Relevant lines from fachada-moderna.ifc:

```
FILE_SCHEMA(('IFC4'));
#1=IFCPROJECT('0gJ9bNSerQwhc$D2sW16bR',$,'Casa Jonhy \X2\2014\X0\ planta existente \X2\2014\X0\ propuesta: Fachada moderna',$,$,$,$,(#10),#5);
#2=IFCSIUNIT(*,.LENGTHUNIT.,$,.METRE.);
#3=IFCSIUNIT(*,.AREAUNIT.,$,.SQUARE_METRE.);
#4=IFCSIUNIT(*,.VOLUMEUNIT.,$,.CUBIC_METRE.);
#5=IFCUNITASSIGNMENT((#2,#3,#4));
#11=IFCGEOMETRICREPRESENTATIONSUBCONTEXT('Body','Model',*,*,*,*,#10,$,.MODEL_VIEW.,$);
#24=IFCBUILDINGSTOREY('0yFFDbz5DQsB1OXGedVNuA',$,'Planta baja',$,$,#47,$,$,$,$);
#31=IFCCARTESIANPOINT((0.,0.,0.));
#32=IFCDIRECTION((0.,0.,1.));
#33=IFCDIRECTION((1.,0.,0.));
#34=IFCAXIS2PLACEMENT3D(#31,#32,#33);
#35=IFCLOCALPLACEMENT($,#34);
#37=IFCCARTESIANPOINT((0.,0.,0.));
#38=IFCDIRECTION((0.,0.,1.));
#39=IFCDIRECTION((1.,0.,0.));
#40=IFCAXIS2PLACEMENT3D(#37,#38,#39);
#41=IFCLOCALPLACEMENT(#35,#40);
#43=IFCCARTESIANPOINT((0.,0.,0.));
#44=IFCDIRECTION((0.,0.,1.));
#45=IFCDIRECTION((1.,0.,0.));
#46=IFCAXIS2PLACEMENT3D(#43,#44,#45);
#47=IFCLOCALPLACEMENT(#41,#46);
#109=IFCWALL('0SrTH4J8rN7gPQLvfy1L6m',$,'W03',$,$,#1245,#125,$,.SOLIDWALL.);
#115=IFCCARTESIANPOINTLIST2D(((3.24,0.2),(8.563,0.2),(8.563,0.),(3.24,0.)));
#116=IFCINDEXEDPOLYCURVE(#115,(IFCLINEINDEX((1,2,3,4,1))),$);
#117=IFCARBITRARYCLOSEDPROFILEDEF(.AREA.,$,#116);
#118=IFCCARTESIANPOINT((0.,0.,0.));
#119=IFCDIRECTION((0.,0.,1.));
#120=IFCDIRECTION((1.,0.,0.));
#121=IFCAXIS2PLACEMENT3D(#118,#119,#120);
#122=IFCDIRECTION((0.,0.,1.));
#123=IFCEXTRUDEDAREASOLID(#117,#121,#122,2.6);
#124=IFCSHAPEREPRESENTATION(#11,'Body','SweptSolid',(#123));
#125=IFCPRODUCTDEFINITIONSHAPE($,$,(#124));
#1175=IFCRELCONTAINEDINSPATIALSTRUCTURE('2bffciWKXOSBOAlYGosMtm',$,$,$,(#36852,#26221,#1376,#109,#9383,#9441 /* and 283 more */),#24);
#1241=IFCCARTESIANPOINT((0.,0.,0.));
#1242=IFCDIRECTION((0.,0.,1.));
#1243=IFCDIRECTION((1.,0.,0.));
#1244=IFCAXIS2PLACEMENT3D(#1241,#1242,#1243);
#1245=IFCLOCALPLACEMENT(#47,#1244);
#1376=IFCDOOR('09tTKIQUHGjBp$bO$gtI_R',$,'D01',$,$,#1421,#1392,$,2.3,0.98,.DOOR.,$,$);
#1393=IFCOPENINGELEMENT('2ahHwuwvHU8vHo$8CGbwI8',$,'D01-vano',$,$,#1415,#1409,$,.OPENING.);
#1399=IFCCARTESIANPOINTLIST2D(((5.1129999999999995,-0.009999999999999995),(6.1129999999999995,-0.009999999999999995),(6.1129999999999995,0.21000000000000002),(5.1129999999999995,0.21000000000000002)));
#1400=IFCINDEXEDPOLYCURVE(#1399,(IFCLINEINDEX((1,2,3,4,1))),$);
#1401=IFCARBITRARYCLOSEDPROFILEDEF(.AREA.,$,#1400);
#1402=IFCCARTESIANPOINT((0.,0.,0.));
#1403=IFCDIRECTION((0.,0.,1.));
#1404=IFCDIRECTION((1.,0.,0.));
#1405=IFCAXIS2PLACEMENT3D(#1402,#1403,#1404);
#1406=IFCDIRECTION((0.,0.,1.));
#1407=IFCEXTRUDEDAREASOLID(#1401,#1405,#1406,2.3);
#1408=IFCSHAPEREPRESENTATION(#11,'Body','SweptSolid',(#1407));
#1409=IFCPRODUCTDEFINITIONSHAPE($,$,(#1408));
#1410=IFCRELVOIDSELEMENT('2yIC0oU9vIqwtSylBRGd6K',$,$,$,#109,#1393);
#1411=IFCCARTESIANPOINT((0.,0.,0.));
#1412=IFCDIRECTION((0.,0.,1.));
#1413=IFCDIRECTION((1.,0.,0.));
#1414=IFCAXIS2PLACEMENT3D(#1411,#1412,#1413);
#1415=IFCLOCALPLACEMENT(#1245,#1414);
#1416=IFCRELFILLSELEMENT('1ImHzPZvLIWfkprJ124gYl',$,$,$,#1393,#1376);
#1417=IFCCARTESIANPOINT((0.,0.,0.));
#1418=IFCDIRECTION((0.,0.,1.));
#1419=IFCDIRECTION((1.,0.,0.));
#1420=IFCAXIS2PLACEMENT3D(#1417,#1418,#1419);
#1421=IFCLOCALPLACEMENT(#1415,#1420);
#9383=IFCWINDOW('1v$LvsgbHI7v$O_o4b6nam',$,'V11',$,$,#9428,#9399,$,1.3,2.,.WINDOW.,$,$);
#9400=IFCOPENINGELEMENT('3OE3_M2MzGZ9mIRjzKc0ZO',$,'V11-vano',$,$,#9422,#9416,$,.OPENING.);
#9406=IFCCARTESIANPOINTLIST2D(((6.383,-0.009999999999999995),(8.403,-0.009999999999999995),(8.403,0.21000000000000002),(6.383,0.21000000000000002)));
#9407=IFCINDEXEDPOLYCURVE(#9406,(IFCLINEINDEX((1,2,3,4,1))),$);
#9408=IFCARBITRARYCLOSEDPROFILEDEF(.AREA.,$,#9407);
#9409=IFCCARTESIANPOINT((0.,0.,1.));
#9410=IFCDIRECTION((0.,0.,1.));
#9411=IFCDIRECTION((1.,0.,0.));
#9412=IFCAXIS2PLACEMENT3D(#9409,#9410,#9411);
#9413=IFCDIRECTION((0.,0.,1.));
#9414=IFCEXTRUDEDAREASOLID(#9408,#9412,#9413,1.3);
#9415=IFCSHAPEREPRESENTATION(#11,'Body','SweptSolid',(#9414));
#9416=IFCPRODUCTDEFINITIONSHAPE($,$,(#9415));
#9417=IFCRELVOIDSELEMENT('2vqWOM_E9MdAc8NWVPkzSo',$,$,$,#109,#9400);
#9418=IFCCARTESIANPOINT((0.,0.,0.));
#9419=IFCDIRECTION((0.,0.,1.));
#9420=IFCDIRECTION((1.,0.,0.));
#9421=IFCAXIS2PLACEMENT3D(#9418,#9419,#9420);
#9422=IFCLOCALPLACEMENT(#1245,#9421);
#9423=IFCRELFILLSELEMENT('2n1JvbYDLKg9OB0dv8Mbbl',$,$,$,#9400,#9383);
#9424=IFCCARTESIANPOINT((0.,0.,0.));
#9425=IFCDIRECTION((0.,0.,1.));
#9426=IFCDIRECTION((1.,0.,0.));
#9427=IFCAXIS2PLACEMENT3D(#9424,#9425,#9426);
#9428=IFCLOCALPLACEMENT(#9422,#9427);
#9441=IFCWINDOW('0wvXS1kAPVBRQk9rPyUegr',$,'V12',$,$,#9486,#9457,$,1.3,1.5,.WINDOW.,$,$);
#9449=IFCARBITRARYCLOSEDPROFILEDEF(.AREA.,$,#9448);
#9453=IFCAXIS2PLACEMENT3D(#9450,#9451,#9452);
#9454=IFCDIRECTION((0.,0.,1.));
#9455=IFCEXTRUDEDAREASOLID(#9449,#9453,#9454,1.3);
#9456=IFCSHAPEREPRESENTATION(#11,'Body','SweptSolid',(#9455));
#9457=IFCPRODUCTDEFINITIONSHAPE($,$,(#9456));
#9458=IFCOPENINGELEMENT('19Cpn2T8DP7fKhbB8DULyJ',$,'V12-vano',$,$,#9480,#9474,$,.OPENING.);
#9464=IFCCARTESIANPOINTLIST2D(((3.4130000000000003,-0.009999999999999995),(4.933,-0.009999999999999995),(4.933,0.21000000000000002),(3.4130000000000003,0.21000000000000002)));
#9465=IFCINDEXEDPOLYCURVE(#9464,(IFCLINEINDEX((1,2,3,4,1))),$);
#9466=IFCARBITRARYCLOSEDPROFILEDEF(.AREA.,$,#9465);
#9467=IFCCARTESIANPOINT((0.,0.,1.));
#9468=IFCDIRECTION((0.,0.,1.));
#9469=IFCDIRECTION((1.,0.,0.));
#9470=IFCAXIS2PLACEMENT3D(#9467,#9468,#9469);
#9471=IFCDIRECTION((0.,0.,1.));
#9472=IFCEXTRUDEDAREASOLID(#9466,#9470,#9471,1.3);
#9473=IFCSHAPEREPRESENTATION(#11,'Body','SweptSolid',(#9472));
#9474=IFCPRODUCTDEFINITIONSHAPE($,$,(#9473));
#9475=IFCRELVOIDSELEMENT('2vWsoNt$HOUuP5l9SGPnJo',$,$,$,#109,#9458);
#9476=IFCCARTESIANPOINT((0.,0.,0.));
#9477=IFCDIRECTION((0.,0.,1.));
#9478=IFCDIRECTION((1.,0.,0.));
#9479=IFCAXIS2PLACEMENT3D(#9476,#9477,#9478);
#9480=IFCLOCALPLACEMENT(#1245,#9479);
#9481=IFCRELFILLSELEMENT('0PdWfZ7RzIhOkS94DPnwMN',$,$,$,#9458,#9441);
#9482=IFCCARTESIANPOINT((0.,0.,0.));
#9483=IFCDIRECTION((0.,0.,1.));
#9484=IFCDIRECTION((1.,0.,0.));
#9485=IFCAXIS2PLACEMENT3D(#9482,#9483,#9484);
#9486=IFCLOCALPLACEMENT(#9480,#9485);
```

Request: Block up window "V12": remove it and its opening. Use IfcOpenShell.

```python
import ifcopenshell
import ifcopenshell.api.feature
import ifcopenshell.api.root
import ifcopenshell.geom
import ifcopenshell.util.shape

model = ifcopenshell.open("fachada-moderna.ifc")
settings = ifcopenshell.geom.settings()


def volume(element):
    """Net volume in cubic metres, openings subtracted."""
    shape = ifcopenshell.geom.create_shape(settings, element)
    return ifcopenshell.util.shape.get_volume(shape.geometry)


window = model.by_id(9441)
opening = window.FillsVoids[0].RelatingOpeningElement
wall = opening.VoidsElements[0].RelatingBuildingElement
before = volume(wall)

ifcopenshell.api.root.remove_product(model, product=window)
ifcopenshell.api.feature.remove_feature(model, feature=opening)

after = volume(wall)

print(f"wall volume {before:.3f} -> {after:.3f} m3")

model.write("fachada-moderna_v2.ifc")
```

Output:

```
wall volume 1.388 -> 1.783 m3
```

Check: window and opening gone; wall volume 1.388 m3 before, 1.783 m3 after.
